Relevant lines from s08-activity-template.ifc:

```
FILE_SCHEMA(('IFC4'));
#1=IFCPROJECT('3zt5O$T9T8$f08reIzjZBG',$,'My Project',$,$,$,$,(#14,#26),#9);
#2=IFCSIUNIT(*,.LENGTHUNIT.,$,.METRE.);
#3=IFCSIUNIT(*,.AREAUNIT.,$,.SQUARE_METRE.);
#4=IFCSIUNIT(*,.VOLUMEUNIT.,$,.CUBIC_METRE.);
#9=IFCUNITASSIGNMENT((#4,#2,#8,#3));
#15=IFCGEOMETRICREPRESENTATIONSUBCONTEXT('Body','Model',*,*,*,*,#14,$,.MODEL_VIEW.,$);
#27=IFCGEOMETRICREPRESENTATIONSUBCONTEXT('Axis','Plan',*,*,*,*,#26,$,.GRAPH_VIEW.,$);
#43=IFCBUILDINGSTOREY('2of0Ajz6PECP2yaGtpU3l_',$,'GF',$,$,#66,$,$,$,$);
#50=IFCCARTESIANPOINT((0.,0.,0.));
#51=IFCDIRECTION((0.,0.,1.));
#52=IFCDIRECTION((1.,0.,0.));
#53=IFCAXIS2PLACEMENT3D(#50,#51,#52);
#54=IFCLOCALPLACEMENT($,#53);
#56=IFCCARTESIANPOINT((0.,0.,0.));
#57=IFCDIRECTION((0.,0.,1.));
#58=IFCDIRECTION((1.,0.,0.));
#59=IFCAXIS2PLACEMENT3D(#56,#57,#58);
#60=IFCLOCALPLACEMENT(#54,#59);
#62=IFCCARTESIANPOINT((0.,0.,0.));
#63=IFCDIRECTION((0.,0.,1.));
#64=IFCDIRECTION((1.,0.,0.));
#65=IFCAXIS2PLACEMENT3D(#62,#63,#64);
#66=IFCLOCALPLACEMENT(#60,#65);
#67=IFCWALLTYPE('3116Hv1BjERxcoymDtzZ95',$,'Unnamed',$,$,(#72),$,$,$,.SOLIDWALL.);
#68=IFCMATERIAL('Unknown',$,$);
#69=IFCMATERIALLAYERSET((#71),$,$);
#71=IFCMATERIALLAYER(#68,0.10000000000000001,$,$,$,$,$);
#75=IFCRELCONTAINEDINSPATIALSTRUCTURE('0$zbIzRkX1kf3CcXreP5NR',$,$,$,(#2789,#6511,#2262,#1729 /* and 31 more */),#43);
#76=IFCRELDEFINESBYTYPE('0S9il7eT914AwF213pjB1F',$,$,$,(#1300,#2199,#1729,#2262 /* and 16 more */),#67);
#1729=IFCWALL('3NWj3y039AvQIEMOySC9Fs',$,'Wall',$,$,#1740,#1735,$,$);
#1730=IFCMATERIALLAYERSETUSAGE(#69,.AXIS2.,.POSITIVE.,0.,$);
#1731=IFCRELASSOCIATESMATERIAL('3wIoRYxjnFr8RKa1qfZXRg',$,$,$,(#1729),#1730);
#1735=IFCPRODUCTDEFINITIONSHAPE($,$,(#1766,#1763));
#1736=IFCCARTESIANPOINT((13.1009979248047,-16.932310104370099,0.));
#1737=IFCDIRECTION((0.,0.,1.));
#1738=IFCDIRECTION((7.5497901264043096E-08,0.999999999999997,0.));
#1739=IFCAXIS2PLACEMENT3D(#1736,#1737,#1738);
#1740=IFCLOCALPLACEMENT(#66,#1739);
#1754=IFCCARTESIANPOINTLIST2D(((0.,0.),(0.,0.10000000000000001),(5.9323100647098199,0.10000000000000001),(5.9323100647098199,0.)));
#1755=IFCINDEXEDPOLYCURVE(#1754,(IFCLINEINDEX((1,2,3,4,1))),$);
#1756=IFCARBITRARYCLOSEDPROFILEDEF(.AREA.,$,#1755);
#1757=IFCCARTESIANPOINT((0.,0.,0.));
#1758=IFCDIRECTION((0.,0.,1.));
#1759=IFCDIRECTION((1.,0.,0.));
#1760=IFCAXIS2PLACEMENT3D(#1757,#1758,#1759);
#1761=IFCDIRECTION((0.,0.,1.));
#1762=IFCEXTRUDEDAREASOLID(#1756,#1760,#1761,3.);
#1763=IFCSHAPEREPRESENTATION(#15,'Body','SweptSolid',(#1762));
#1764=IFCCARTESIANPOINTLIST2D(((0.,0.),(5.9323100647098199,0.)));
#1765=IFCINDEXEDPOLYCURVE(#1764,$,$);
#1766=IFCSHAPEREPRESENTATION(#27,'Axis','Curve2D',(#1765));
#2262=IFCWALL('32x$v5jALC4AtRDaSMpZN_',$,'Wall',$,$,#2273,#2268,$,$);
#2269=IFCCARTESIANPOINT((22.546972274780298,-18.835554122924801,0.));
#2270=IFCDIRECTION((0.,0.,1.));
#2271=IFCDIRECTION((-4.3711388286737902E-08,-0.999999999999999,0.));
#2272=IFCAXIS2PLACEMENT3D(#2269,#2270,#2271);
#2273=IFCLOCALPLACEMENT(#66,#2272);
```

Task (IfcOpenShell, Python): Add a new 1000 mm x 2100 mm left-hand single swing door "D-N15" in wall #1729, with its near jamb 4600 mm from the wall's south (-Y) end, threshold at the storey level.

```python
import numpy as np
import ifcopenshell
import ifcopenshell.api.feature
import ifcopenshell.api.geometry
import ifcopenshell.api.root
import ifcopenshell.api.spatial
import ifcopenshell.geom
import ifcopenshell.util.element
import ifcopenshell.util.placement
import ifcopenshell.util.representation
import ifcopenshell.util.shape
import ifcopenshell.util.unit

model = ifcopenshell.open("s08-activity-template.ifc")
unit_scale = ifcopenshell.util.unit.calculate_unit_scale(model)
settings = ifcopenshell.geom.settings()


def volume(element):
    """Net volume in cubic metres, openings subtracted."""
    shape = ifcopenshell.geom.create_shape(settings, element)
    return ifcopenshell.util.shape.get_volume(shape.geometry)


wall = model.by_guid("3NWj3y039AvQIEMOySC9Fs")
storey = ifcopenshell.util.element.get_container(wall, ifc_class="IfcBuildingStorey")
context = ifcopenshell.util.representation.get_context(model, "Model", "Body", "MODEL_VIEW")
before = volume(wall)

width, height, from_end, sill = 1, 2.1, 4.6, 0.0  # metres

# The wall runs along its own X axis, and the end named is its -X end.
wall_shape = ifcopenshell.geom.create_shape(settings, wall)
x, y, z = ifcopenshell.util.shape.get_vertices(wall_shape.geometry).T
start = x.min() + from_end
face, thickness = float(y.min()), float(y.max() - y.min())
wall_matrix = ifcopenshell.util.placement.get_local_placement(wall.ObjectPlacement)
level = ifcopenshell.util.placement.get_local_placement(storey.ObjectPlacement)[2, 3]


def in_wall(x, y):
    """Placement at x, y metres in the wall's axes, at sill height."""
    matrix = wall_matrix.copy()
    matrix[:, 3] = wall_matrix @ np.array([x / unit_scale, y / unit_scale, 0.0, 1.0])
    matrix[2, 3] = level + sill / unit_scale
    return matrix


# Opening: a box that overshoots both wall faces by 50 mm.
opening = ifcopenshell.api.root.create_entity(model, ifc_class="IfcOpeningElement", predefined_type="OPENING")
box = ifcopenshell.api.geometry.add_wall_representation(
    model, context=context, length=width, height=height, thickness=thickness + 0.1
)
ifcopenshell.api.geometry.assign_representation(model, product=opening, representation=box)
ifcopenshell.api.geometry.edit_object_placement(model, product=opening, matrix=in_wall(start, face - 0.05), is_si=False)
ifcopenshell.api.feature.add_feature(model, feature=opening, element=wall)

door = ifcopenshell.api.root.create_entity(model, ifc_class="IfcDoor", name="D-N15", predefined_type="DOOR")
door.OverallWidth, door.OverallHeight = width / unit_scale, height / unit_scale
door.OperationType = "SINGLE_SWING_LEFT"
body = ifcopenshell.api.geometry.add_door_representation(
    model,
    context=context,
    overall_width=door.OverallWidth,
    overall_height=door.OverallHeight,
    operation_type="SINGLE_SWING_LEFT",
    lining_properties={"LiningDepth": thickness / unit_scale, "ThresholdDepth": thickness / unit_scale},
)
ifcopenshell.api.geometry.assign_representation(model, product=door, representation=body)
ifcopenshell.api.spatial.assign_container(model, products=[door], relating_structure=storey)
ifcopenshell.api.feature.add_filling(model, opening=opening, element=door)

# The lining spans the wall, so the door starts at the wall face.
ifcopenshell.api.geometry.edit_object_placement(model, product=door, matrix=in_wall(start, face), is_si=False)

after = volume(wall)

print(f"wall volume {before:.3f} -> {after:.3f} m3")

model.write("s08-activity-template_updated.ifc")
```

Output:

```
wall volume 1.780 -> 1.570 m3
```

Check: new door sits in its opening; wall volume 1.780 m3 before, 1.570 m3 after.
